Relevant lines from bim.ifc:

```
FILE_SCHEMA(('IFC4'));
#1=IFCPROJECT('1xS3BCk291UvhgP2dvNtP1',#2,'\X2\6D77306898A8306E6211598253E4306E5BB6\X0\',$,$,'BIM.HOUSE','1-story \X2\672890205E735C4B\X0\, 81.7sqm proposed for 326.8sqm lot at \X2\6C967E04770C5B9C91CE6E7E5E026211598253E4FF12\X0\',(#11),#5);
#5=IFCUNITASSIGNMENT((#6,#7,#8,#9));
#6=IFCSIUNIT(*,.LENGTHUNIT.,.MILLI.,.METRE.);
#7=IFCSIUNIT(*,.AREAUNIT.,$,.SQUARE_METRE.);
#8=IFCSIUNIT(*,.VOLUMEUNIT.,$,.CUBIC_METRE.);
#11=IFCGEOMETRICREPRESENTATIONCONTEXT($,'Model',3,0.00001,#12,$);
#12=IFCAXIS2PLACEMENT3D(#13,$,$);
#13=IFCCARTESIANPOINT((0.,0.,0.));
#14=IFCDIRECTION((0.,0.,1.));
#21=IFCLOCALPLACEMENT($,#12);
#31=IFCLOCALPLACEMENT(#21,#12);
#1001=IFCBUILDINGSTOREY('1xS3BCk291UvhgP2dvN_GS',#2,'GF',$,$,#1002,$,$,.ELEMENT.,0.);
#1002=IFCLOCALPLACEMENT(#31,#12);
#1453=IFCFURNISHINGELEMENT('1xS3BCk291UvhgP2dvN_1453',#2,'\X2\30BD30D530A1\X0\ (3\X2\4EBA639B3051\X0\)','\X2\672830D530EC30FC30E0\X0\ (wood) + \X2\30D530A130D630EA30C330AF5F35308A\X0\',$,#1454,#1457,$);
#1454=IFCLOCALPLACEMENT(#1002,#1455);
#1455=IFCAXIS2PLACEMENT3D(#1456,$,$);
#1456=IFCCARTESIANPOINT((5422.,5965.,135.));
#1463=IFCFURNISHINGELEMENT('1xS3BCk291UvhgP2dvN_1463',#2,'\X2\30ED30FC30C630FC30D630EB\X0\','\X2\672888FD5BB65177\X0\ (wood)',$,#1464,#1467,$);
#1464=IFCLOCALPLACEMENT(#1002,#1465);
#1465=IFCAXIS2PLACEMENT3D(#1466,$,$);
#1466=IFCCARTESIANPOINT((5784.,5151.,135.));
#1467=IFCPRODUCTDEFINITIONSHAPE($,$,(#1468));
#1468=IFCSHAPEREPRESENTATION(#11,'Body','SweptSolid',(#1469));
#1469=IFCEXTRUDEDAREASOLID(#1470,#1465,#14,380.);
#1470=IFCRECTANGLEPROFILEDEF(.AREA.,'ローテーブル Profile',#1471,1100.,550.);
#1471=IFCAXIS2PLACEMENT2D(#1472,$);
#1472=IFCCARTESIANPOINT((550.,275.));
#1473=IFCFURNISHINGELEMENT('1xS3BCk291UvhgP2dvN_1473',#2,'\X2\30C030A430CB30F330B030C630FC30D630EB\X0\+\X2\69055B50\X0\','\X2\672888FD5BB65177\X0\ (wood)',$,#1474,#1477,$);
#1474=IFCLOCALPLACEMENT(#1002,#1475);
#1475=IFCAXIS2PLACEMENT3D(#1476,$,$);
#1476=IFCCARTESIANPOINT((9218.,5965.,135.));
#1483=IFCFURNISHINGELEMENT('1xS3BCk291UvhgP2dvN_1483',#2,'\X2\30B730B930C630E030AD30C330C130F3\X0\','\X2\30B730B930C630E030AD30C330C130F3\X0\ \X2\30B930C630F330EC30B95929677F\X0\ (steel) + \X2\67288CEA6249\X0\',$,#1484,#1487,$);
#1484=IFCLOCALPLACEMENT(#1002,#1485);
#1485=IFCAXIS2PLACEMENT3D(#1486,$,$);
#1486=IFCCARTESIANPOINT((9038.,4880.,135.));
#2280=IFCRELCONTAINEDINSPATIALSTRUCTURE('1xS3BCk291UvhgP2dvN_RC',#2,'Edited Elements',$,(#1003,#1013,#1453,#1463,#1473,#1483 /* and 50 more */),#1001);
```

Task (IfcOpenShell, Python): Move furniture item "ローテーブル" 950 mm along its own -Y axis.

```python
import ifcopenshell
import ifcopenshell.api.geometry
import ifcopenshell.util.placement

model = ifcopenshell.open("bim.ifc")

item = model.by_id(1463)
matrix = ifcopenshell.util.placement.get_local_placement(item.ObjectPlacement)
matrix[:3, 3] -= matrix[:3, 1] * 950.0
ifcopenshell.api.geometry.edit_object_placement(model, product=item, matrix=matrix, is_si=False)

print(ifcopenshell.util.placement.get_local_placement(item.ObjectPlacement).round(3) + 0.0)

model.write("bim_updated.ifc")
```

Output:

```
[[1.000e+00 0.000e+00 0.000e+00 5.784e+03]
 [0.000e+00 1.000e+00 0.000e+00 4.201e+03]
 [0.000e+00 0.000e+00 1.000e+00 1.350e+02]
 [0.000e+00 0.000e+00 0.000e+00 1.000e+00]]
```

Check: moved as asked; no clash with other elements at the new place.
